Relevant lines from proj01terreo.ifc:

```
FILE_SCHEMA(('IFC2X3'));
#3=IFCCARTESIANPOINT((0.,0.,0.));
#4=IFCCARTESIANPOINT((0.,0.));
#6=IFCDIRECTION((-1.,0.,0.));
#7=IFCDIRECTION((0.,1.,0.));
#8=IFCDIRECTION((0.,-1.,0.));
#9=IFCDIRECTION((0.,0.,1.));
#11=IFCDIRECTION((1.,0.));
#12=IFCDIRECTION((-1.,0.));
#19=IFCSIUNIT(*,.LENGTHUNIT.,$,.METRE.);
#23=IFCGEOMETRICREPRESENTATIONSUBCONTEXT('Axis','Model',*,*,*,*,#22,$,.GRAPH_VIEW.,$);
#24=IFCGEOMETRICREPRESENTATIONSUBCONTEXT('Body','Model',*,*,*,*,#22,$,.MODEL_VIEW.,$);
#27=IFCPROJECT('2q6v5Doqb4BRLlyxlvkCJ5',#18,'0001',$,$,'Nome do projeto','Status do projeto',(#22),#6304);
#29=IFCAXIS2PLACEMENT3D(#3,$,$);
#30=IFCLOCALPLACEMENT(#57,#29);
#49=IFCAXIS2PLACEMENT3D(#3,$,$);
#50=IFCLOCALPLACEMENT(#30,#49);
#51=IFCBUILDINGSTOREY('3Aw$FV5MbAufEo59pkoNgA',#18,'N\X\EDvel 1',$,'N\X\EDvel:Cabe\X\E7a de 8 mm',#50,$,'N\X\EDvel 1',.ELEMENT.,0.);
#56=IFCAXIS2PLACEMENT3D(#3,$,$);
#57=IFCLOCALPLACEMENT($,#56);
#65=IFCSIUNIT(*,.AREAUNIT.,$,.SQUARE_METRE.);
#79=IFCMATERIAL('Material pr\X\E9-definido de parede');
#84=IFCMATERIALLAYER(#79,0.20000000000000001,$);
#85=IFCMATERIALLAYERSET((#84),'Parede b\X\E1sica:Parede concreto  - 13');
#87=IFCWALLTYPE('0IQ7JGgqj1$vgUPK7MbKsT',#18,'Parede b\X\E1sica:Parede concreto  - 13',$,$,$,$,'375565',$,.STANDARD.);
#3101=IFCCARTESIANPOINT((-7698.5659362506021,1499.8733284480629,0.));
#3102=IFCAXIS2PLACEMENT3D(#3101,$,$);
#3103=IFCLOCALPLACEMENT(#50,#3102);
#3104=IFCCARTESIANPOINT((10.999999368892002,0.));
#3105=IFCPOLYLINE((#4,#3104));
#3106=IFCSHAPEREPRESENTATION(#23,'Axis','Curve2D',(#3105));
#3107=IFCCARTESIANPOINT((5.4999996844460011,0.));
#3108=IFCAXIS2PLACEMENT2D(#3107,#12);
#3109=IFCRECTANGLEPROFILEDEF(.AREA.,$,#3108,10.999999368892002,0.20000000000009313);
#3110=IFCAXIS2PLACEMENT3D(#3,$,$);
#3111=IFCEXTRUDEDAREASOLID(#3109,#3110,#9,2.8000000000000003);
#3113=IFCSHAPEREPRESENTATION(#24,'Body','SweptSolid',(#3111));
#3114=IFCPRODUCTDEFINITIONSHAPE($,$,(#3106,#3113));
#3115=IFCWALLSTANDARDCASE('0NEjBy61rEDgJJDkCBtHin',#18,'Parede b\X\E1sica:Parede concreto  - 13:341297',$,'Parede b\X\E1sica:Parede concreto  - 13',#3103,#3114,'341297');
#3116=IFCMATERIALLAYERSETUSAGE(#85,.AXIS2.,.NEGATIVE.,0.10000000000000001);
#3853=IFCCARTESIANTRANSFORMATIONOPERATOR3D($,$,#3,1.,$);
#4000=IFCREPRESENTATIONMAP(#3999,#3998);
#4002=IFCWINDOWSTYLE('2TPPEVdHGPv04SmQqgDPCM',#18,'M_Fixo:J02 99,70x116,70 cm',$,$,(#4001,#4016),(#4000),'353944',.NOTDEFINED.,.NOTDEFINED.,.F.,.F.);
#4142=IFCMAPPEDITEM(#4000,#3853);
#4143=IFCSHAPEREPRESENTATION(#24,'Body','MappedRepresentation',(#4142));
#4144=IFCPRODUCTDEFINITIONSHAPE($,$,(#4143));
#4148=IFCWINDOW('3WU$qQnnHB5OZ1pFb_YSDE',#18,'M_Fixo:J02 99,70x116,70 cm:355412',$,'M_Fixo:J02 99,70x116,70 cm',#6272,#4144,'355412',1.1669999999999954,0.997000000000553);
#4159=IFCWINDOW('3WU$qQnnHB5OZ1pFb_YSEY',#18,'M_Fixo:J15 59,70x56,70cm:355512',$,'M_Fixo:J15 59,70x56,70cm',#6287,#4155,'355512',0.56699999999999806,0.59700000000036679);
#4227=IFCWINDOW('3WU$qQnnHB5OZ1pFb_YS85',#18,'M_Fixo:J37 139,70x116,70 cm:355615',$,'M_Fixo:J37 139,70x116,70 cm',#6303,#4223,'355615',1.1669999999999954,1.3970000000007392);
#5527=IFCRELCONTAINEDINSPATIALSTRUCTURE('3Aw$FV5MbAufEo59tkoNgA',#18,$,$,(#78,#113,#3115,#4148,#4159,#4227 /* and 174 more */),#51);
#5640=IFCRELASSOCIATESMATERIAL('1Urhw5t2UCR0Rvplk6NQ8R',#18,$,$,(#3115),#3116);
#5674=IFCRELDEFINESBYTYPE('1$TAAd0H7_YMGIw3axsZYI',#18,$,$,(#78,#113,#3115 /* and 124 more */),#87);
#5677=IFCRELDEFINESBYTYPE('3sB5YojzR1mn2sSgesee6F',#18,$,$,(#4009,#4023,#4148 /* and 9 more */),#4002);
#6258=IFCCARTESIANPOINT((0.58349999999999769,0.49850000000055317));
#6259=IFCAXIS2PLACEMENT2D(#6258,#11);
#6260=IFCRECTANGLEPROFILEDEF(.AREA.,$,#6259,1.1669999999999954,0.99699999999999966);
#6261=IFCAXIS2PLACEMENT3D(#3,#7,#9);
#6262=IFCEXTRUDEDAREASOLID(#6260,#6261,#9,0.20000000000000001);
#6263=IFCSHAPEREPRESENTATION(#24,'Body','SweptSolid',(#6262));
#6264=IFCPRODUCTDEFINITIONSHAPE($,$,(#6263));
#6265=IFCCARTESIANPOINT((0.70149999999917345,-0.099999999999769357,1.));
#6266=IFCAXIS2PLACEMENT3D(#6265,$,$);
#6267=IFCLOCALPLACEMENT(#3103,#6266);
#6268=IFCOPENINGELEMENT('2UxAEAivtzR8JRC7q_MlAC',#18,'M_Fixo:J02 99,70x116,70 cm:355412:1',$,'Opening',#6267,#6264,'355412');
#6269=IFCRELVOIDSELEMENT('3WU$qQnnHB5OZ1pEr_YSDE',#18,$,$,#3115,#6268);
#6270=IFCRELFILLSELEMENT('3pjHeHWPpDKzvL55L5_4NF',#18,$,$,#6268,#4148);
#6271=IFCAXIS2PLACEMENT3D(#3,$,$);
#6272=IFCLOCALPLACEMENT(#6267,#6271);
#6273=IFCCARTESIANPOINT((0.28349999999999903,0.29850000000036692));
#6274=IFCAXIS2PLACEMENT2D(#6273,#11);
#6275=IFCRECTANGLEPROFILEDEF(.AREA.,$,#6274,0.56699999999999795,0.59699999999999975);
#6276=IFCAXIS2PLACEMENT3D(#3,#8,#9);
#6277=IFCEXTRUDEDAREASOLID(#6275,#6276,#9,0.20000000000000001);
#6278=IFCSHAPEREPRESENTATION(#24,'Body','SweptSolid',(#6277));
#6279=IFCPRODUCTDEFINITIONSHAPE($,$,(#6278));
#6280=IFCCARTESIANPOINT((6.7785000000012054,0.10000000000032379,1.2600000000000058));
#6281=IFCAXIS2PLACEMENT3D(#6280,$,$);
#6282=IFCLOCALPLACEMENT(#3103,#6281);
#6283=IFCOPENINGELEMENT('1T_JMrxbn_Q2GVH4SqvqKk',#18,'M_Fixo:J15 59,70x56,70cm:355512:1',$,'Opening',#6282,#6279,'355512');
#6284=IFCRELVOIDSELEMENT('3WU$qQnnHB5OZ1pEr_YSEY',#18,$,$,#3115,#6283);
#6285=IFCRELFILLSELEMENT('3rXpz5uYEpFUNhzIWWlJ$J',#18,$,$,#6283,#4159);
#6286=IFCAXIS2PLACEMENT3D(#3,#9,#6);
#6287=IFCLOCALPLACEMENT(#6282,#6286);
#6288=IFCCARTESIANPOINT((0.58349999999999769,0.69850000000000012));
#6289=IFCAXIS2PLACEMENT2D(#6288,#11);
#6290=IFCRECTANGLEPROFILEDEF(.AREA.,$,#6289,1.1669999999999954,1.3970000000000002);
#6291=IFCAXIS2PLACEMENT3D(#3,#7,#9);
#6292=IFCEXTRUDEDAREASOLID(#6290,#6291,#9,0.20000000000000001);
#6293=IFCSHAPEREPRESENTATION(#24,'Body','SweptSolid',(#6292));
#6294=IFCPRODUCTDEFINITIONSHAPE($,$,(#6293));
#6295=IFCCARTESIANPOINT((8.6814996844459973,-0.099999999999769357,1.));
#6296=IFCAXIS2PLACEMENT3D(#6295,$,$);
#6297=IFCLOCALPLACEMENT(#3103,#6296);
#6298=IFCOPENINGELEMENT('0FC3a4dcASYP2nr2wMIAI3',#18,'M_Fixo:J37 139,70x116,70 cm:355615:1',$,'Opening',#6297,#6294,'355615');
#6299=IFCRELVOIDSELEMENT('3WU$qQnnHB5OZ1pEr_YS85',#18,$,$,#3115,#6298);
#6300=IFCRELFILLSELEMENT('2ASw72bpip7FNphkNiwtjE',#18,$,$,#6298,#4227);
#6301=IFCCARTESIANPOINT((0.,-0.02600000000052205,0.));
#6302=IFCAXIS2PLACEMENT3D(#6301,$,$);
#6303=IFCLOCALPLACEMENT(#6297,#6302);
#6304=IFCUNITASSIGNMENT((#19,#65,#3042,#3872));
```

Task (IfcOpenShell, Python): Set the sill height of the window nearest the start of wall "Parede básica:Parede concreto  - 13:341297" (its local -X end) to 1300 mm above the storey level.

```python
import numpy as np
import ifcopenshell
import ifcopenshell.api.geometry
import ifcopenshell.geom
import ifcopenshell.util.element
import ifcopenshell.util.placement
import ifcopenshell.util.shape
import ifcopenshell.util.unit

model = ifcopenshell.open("proj01terreo.ifc")
unit_scale = ifcopenshell.util.unit.calculate_unit_scale(model)

window = model.by_guid("3WU$qQnnHB5OZ1pFb_YSDE")
opening = window.FillsVoids[0].RelatingOpeningElement
storey = ifcopenshell.util.element.get_container(window, ifc_class="IfcBuildingStorey")
level = ifcopenshell.util.placement.get_local_placement(storey.ObjectPlacement)[2, 3]

# The opening's origin need not be at the sill, so measure its lowest point.
shape = ifcopenshell.geom.create_shape(ifcopenshell.geom.settings(), opening)
bottom = ifcopenshell.util.shape.get_shape_bottom_elevation(shape, shape.geometry) / unit_scale
dz = level + 1.3 - bottom

shift = np.array([0.0, 0.0, dz])
# The window is placed relative to its opening, so it follows when the opening moves.
matrix = ifcopenshell.util.placement.get_local_placement(opening.ObjectPlacement)
matrix[:3, 3] += shift
ifcopenshell.api.geometry.edit_object_placement(
    model, product=opening, matrix=matrix, is_si=False, should_transform_children=True
)

print(f"moved by {dz * unit_scale:+.3f} m")

model.write("proj01terreo-out.ifc")
```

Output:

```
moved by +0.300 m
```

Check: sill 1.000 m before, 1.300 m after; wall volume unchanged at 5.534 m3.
